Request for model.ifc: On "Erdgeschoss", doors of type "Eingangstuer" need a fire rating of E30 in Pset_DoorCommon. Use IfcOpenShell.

First a look at what the model holds.

```python
import ifcopenshell
import ifcopenshell.util.element

model = ifcopenshell.open("model.ifc")
print(model.schema)
storey = next(s for s in model.by_type("IfcBuildingStorey") if s.Name == "Erdgeschoss")
doors = [e for e in ifcopenshell.util.element.get_decomposition(storey) if e.is_a("IfcDoor")]
seen = {}
for e in doors:
    element_type = ifcopenshell.util.element.get_type(e)
    key = (element_type.Name if element_type != e and element_type else None, ifcopenshell.util.element.get_pset(e, "Pset_DoorCommon", "FireRating"))
    seen[key] = seen.get(key, 0) + 1
for (name, value), count in sorted(seen.items(), key=str):
    print(count, "x", name, "|", value)
```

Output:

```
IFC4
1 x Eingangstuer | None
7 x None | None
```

```python
import ifcopenshell
import ifcopenshell.api.pset
import ifcopenshell.util.element

model = ifcopenshell.open("model.ifc")

storey = next(s for s in model.by_type("IfcBuildingStorey") if s.Name == "Erdgeschoss")
doors = [e for e in ifcopenshell.util.element.get_decomposition(storey) if e.is_a("IfcDoor")]

count = 0
for e in doors:
    element_type = ifcopenshell.util.element.get_type(e)
    if element_type in (None, e) or element_type.Name != "Eingangstuer":
        continue
    # add_pset returns the element's existing set when there is one.
    pset = ifcopenshell.api.pset.add_pset(model, product=e, name="Pset_DoorCommon")
    ifcopenshell.api.pset.edit_pset(model, pset=pset, properties={"FireRating": "E30"})
    count += 1

print(count, "doors updated")

model.write("model_edited.ifc")
```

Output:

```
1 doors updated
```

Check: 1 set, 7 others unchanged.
